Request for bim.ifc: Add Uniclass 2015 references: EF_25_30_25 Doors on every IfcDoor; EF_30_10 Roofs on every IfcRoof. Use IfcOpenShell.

First a look at what the model holds.

```python
import ifcopenshell

model = ifcopenshell.open("bim.ifc")
print(model.schema)
print("classifications:", [c.Name for c in model.by_type("IfcClassification")])
for ifc_class in ("IfcDoor", "IfcRoof", "IfcStair", "IfcWall", "IfcWindow"):
    print(ifc_class, len(model.by_type(ifc_class)))
```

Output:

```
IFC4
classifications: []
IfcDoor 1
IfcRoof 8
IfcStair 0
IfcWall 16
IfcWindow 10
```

```python
import ifcopenshell
import ifcopenshell.api.classification

model = ifcopenshell.open("bim.ifc")

system = ifcopenshell.api.classification.add_classification(model, classification="Uniclass 2015")

codes = {
    "IfcDoor": ("EF_25_30_25", "Doors"),
    "IfcRoof": ("EF_30_10", "Roofs"),
}
for ifc_class, (code, name) in codes.items():
    products = model.by_type(ifc_class)
    ifcopenshell.api.classification.add_reference(
        model, products=products, classification=system, identification=code, name=name
    )
    print(code, len(products))

model.write("bim_updated.ifc")
```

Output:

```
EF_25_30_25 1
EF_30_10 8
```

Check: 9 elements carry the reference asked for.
